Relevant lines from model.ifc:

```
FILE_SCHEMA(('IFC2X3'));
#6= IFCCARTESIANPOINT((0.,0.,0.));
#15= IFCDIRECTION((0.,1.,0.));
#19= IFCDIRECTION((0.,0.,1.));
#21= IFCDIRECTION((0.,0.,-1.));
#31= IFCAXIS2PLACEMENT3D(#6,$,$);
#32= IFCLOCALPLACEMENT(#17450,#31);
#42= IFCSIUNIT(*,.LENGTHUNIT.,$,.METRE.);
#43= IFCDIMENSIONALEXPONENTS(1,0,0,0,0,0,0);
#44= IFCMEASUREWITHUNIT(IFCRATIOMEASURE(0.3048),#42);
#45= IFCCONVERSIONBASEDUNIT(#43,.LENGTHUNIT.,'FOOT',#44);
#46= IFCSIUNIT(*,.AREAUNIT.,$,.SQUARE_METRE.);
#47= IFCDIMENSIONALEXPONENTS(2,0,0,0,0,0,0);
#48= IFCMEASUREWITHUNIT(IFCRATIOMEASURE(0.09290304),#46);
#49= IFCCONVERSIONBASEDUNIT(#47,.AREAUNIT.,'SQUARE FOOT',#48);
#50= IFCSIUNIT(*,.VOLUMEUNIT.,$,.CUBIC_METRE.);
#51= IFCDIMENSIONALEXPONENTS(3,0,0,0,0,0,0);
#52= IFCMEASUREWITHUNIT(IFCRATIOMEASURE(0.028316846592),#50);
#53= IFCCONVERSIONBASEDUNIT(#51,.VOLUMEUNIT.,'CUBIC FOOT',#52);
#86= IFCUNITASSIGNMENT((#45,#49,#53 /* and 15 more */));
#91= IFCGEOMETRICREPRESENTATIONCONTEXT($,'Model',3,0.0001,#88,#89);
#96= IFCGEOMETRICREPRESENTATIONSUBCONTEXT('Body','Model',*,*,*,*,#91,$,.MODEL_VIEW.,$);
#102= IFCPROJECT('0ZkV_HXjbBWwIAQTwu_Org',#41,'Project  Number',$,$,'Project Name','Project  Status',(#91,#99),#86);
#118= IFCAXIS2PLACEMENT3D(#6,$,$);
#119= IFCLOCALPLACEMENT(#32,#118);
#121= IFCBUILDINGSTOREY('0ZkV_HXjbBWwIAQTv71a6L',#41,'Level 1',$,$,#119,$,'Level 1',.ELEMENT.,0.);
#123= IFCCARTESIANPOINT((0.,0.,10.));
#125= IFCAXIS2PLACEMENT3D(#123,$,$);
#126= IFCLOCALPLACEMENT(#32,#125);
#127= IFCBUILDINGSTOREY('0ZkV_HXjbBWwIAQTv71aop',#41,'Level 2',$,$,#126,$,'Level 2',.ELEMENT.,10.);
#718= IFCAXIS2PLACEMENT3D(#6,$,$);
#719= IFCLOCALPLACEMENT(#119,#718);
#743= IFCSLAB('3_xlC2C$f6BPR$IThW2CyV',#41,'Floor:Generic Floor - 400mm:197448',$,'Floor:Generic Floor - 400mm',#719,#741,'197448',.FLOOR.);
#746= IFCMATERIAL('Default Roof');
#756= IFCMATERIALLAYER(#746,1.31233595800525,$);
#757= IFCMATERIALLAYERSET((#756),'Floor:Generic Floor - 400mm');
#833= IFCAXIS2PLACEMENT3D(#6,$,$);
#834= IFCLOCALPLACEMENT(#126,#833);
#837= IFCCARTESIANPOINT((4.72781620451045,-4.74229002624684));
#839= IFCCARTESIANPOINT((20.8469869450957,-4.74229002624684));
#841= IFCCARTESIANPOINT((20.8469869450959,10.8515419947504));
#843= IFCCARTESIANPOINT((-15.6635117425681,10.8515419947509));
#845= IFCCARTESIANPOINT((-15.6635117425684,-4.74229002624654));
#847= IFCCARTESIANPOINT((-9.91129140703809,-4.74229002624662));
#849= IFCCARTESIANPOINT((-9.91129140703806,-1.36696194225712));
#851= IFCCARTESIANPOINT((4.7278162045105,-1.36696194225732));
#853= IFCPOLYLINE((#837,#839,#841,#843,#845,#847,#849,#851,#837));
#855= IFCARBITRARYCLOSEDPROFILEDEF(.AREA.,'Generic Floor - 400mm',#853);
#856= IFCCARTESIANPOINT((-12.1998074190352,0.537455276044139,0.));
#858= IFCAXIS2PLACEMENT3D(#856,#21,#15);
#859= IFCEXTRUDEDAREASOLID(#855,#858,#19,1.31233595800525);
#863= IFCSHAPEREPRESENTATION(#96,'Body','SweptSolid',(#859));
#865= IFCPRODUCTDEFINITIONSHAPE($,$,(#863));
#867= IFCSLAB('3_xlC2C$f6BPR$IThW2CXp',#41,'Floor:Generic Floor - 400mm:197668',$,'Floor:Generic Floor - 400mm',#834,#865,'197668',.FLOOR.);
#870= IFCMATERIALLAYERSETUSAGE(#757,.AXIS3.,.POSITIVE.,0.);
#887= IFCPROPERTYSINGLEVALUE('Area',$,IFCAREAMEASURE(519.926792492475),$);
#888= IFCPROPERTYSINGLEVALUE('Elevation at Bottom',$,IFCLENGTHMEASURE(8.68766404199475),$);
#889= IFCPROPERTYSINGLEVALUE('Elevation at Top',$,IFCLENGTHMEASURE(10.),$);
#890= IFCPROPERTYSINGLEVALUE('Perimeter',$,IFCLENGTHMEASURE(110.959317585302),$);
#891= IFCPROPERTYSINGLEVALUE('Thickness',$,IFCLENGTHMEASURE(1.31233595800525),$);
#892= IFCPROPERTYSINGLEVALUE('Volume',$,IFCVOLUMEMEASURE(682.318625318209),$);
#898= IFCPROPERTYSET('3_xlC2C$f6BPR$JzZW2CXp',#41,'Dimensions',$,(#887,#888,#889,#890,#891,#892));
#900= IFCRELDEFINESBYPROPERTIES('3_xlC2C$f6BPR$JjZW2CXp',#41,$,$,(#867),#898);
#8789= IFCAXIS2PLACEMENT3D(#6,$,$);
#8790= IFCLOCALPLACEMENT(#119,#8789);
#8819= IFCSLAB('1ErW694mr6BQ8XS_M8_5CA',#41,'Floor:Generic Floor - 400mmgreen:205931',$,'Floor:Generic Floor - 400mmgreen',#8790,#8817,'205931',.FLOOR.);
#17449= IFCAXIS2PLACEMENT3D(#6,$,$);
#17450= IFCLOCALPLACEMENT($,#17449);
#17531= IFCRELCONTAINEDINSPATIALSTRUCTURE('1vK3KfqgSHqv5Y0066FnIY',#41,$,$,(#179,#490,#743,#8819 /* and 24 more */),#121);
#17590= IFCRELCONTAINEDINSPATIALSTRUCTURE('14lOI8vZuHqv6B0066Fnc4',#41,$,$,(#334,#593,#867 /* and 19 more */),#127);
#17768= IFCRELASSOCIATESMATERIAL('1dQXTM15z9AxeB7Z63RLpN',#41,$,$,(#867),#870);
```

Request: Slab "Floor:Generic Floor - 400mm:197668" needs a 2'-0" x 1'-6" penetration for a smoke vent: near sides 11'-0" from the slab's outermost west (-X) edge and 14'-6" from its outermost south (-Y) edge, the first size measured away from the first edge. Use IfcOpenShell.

```python
import numpy as np
import ifcopenshell
import ifcopenshell.api.feature
import ifcopenshell.api.geometry
import ifcopenshell.api.pset
import ifcopenshell.api.root
import ifcopenshell.geom
import ifcopenshell.util.element
import ifcopenshell.util.placement
import ifcopenshell.util.representation
import ifcopenshell.util.shape
import ifcopenshell.util.unit

model = ifcopenshell.open("model.ifc")
unit_scale = ifcopenshell.util.unit.calculate_unit_scale(model)
area_scale = ifcopenshell.util.unit.calculate_unit_scale(model, "AREAUNIT")
volume_scale = ifcopenshell.util.unit.calculate_unit_scale(model, "VOLUMEUNIT")
settings = ifcopenshell.geom.settings()


def volume(element):
    """Net volume in cubic metres, openings subtracted."""
    shape = ifcopenshell.geom.create_shape(settings, element)
    return ifcopenshell.util.shape.get_volume(shape.geometry)


slab = model.by_guid("3_xlC2C$f6BPR$IThW2CXp")
before = volume(slab)

# Extent in the slab's own axes, in metres. The edges named are its -X and -Y sides.
slab_shape = ifcopenshell.geom.create_shape(settings, slab)
vertices = ifcopenshell.util.shape.get_vertices(slab_shape.geometry)
x_min, y_min, bottom = vertices.min(axis=0)
top = vertices[:, 2].max()

opening = ifcopenshell.api.root.create_entity(model, ifc_class="IfcOpeningElement", name="Smoke vent opening")
context = ifcopenshell.util.representation.get_context(model, "Model", "Body", "MODEL_VIEW")
width, depth = 0.6096, 0.4572
outline = [(0.0, 0.0), (width, 0.0), (width, depth), (0.0, depth), (0.0, 0.0)]
# Overshoot both faces by 50 mm so the cut is clean.
shape = ifcopenshell.api.geometry.add_slab_representation(
    model, context=context, depth=top - bottom + 0.1, polyline=outline
)
ifcopenshell.api.geometry.assign_representation(model, product=opening, representation=shape)

matrix = ifcopenshell.util.placement.get_local_placement(slab.ObjectPlacement)
matrix[:, 3] = matrix @ np.append(np.array([x_min + 3.3528, y_min + 4.4196, bottom - 0.05]) / unit_scale, 1.0)
ifcopenshell.api.geometry.edit_object_placement(model, product=opening, matrix=matrix, is_si=False)
ifcopenshell.api.feature.add_feature(model, feature=opening, element=slab)

after = volume(slab)

# Update the slab's stored quantities.
pset = model.by_id(ifcopenshell.util.element.get_pset(slab, "Dimensions", should_inherit=False)["id"])
ifcopenshell.api.pset.edit_pset(model, pset=pset, properties={
    "Area": model.create_entity("IfcAreaMeasure", after / (top - bottom) / area_scale),
    "Volume": model.create_entity("IfcVolumeMeasure", after / volume_scale),
})

print(f"slab volume {before:.3f} -> {after:.3f} m3")

model.write("model_edited.ifc")
```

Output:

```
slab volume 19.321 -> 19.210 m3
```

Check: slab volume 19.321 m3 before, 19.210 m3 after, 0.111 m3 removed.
